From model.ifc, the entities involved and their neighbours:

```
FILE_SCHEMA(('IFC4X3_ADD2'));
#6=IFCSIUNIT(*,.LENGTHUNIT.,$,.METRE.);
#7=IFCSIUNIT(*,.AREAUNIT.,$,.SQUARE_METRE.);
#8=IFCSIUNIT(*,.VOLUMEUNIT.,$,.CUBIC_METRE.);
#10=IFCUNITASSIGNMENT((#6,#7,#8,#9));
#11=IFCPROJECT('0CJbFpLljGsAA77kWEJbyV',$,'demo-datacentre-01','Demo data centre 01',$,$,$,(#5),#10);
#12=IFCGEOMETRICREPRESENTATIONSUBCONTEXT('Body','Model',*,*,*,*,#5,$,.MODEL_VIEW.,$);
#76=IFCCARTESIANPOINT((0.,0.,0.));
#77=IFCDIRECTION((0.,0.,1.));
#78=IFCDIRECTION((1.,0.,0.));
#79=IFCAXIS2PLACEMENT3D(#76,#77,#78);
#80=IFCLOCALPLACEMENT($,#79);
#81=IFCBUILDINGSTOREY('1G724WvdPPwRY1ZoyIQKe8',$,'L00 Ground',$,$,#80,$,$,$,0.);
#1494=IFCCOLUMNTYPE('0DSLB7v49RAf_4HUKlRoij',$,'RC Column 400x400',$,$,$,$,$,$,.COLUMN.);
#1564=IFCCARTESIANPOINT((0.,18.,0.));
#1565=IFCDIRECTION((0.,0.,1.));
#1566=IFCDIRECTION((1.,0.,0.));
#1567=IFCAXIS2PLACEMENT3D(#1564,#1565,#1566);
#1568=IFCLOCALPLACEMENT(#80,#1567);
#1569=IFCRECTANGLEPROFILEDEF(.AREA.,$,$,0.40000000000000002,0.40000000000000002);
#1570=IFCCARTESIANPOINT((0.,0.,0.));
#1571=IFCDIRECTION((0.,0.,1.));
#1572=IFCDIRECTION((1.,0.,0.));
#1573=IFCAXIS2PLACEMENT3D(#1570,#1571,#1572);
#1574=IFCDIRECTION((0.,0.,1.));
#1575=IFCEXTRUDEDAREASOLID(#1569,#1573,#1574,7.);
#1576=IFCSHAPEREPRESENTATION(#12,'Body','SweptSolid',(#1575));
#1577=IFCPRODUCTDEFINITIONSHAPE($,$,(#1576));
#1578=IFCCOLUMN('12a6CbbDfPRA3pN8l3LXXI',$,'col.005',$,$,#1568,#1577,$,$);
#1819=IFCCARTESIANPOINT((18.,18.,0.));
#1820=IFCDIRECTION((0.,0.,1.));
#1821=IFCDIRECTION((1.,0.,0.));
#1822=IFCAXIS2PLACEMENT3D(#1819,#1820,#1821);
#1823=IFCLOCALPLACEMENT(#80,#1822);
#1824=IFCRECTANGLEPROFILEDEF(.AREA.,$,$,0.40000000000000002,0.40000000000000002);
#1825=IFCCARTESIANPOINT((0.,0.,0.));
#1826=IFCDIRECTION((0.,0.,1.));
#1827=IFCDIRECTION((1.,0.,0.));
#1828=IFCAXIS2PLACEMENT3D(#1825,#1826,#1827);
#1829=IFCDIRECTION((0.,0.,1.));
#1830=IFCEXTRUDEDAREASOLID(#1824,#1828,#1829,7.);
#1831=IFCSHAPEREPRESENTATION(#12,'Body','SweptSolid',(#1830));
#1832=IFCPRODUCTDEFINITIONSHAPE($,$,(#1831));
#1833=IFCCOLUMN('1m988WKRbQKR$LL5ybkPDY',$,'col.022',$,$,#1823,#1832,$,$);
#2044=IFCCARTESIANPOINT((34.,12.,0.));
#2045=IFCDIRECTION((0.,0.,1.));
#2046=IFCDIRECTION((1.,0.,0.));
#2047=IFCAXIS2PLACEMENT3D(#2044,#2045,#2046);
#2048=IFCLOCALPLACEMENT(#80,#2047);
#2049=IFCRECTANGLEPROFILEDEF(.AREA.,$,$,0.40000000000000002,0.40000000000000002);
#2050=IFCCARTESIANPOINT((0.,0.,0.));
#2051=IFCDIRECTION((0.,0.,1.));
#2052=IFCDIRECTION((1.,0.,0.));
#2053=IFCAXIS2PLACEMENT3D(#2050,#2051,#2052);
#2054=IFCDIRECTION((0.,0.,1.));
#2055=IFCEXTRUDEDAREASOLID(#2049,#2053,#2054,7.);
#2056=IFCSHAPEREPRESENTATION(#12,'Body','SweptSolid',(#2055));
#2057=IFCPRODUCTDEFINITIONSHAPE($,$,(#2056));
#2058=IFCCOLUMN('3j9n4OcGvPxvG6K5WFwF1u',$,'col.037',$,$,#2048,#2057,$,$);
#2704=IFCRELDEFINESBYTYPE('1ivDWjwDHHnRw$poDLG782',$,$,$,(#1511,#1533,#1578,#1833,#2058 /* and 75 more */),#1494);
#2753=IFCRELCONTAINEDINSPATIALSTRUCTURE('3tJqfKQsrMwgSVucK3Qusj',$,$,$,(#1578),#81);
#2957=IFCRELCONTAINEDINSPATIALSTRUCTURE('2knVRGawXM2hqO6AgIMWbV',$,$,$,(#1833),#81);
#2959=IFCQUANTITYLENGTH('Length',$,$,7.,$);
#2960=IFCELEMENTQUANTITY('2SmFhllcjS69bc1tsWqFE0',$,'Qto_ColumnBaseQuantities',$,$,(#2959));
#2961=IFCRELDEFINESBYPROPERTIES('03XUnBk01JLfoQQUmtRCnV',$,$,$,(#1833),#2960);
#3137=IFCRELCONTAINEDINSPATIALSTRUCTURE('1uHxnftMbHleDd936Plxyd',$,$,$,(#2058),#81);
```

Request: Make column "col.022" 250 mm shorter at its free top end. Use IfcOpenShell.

```python
import ifcopenshell
import ifcopenshell.api.pset
import ifcopenshell.util.element
import ifcopenshell.util.representation
import ifcopenshell.util.unit

model = ifcopenshell.open("model.ifc")
unit_scale = ifcopenshell.util.unit.calculate_unit_scale(model)

member = model.by_guid("1m988WKRbQKR$LL5ybkPDY")
change = -0.25 / unit_scale

# The extrusion runs towards the end named, so only its depth changes.
body = ifcopenshell.util.representation.get_representation(member, "Model", "Body")
solid = body.Items[0]
old_length = solid.Depth
solid.Depth += change

# Update the stored length and volume.
qto = model.by_id(ifcopenshell.util.element.get_pset(member, "Qto_ColumnBaseQuantities", should_inherit=False)["id"])
ifcopenshell.api.pset.edit_qto(model, qto=qto, properties={"Length": solid.Depth})

print(f"length {old_length:g} -> {solid.Depth:g}")

model.write("model_rev.ifc")
```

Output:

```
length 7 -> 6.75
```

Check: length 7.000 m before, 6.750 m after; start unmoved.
